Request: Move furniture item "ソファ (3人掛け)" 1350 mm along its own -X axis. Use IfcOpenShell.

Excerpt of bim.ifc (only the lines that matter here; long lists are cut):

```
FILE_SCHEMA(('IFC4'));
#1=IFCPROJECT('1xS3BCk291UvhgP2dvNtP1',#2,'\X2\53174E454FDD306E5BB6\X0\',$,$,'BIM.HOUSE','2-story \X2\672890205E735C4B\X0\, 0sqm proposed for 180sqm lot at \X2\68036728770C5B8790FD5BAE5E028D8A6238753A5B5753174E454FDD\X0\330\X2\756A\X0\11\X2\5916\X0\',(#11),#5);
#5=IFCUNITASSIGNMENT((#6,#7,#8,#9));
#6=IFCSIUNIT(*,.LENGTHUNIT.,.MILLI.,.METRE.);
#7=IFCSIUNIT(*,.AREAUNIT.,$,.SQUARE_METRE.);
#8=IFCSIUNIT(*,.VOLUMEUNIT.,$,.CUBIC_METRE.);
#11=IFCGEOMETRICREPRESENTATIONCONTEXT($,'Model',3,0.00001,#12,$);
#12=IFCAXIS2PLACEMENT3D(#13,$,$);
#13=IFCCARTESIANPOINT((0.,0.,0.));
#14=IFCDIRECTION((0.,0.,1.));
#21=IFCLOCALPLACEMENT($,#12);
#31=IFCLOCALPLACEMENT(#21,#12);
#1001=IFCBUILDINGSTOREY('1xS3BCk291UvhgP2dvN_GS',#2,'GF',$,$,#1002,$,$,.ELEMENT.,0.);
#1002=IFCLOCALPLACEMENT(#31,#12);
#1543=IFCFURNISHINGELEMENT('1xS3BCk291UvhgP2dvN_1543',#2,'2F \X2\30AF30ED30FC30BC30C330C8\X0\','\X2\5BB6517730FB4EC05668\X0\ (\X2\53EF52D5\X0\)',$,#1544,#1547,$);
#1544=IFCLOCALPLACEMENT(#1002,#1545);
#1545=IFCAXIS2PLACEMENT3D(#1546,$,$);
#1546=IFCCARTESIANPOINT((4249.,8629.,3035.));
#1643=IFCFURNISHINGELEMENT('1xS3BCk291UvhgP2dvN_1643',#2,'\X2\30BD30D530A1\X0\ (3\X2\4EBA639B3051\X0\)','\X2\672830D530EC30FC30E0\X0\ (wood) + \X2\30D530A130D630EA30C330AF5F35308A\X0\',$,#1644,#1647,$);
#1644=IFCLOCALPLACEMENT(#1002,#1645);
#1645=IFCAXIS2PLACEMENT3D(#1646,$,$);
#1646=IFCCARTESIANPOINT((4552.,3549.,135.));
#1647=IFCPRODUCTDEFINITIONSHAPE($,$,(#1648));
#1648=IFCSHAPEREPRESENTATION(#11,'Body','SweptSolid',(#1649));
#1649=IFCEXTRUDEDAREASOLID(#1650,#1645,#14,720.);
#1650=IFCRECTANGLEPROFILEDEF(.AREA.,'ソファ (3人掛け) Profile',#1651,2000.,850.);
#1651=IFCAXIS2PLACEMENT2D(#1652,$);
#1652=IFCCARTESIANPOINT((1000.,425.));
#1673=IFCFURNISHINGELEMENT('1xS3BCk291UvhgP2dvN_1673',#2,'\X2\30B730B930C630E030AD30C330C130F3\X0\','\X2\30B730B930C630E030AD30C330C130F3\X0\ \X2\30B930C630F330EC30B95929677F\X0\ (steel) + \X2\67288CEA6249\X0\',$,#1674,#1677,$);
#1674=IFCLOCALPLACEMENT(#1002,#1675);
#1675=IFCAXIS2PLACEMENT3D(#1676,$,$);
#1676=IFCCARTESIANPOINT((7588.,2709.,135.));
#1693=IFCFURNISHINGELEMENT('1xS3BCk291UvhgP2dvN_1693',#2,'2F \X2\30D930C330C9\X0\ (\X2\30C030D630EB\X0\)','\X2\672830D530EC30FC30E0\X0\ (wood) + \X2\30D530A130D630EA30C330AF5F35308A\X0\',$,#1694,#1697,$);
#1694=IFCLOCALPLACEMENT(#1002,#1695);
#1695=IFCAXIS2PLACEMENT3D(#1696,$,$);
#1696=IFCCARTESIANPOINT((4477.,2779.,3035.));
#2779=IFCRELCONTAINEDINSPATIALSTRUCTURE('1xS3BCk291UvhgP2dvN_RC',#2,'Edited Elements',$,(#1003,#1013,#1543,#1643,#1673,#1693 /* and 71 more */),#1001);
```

```python
import ifcopenshell
import ifcopenshell.api.geometry
import ifcopenshell.util.placement
import ifcopenshell.util.unit

model = ifcopenshell.open("bim.ifc")
unit_scale = ifcopenshell.util.unit.calculate_unit_scale(model)

item = model.by_guid("1xS3BCk291UvhgP2dvN_1643")
matrix = ifcopenshell.util.placement.get_local_placement(item.ObjectPlacement)
matrix[:3, 3] -= matrix[:3, 0] * 1.35 / unit_scale
ifcopenshell.api.geometry.edit_object_placement(model, product=item, matrix=matrix, is_si=False)

print(ifcopenshell.util.placement.get_local_placement(item.ObjectPlacement).round(3) + 0.0)

model.write("bim_edited.ifc")
```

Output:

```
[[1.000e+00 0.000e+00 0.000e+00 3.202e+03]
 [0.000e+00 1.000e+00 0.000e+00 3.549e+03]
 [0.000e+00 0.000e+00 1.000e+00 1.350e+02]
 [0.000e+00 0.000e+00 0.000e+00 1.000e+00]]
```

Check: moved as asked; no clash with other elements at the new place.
